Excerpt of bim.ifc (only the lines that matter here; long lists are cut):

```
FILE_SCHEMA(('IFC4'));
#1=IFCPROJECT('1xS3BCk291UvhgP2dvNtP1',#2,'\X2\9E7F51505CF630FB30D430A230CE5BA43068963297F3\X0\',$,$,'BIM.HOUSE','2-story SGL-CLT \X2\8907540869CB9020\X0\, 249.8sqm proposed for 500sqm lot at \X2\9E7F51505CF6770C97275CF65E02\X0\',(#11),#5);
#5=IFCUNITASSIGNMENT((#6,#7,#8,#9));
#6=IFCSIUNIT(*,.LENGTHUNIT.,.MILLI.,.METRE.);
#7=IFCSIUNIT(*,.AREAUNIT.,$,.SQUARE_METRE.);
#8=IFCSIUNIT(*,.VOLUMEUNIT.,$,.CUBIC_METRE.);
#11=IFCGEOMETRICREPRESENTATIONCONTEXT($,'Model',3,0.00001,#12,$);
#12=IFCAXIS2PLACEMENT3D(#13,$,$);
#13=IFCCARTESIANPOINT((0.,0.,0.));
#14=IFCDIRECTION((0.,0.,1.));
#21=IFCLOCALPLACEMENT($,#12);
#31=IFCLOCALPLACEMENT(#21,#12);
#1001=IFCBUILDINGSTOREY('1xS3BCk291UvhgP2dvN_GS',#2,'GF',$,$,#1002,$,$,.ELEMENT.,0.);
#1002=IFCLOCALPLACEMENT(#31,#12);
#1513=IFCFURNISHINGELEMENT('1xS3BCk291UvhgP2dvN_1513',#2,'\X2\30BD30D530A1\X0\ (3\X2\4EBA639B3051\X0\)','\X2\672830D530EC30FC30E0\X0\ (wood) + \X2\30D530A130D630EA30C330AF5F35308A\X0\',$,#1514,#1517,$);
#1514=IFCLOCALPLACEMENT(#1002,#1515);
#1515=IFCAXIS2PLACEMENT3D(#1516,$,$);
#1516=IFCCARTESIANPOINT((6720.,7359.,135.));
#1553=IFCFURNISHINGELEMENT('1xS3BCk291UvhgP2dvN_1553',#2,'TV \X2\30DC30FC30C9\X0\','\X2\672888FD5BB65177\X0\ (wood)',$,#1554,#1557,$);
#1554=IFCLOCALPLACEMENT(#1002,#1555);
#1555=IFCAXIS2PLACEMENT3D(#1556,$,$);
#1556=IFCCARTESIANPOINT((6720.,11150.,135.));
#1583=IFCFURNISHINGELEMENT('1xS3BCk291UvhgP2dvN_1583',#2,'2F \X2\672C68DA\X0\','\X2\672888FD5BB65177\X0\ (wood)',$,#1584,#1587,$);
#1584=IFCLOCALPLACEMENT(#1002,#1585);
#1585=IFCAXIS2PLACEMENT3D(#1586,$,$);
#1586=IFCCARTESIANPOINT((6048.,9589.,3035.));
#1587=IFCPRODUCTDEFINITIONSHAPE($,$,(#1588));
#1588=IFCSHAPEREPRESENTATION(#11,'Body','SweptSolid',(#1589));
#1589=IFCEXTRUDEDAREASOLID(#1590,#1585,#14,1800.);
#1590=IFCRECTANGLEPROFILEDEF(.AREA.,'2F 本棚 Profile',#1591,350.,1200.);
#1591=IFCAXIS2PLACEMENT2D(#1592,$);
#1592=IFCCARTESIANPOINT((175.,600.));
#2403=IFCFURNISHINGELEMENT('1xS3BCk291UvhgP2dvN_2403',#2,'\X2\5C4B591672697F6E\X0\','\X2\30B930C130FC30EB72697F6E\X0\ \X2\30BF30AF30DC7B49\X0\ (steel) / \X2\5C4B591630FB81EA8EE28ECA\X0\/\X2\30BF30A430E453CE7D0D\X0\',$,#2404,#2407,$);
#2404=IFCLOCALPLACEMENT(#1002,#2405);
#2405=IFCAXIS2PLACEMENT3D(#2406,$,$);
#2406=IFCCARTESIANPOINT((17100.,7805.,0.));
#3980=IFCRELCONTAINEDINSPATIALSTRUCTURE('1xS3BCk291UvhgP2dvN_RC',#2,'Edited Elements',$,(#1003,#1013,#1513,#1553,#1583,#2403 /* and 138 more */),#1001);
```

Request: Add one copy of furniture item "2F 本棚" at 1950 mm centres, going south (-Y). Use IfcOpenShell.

```python
import numpy as np
import ifcopenshell
import ifcopenshell.api.geometry
import ifcopenshell.api.root
import ifcopenshell.util.element
import ifcopenshell.util.placement
import ifcopenshell.util.unit

model = ifcopenshell.open("bim.ifc")
unit_scale = ifcopenshell.util.unit.calculate_unit_scale(model)


def reuse_history(source, copy):
    """copy_class also copies each property set's owner history, people and application; keep the originals."""
    for rel in copy.IsDefinedBy:
        if rel.is_a("IfcRelDefinesByProperties") and (history := rel.RelatingPropertyDefinition.OwnerHistory):
            rel.RelatingPropertyDefinition.OwnerHistory = source.OwnerHistory
            ifcopenshell.util.element.remove_deep2(model, history)


source = model.by_guid("1xS3BCk291UvhgP2dvN_1583")
base = ifcopenshell.util.placement.get_local_placement(source.ObjectPlacement)
step = np.array([0.0, -1.0, 0.0]) * 1.95 / unit_scale

for i in range(1, 2):
    copy = ifcopenshell.api.root.copy_class(model, product=source)
    copy.Representation = ifcopenshell.util.element.copy_deep(
        model, source.Representation, exclude=["IfcGeometricRepresentationContext", "IfcRepresentationMap"]
    )
    reuse_history(source, copy)
    matrix = base.copy()
    matrix[:3, 3] += i * step
    print("added at", matrix[:3, 3].round(3) + 0.0)
    ifcopenshell.api.geometry.edit_object_placement(model, product=copy, matrix=matrix, is_si=False)

model.write("bim_updated.ifc")
```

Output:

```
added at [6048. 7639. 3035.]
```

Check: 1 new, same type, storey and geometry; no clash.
